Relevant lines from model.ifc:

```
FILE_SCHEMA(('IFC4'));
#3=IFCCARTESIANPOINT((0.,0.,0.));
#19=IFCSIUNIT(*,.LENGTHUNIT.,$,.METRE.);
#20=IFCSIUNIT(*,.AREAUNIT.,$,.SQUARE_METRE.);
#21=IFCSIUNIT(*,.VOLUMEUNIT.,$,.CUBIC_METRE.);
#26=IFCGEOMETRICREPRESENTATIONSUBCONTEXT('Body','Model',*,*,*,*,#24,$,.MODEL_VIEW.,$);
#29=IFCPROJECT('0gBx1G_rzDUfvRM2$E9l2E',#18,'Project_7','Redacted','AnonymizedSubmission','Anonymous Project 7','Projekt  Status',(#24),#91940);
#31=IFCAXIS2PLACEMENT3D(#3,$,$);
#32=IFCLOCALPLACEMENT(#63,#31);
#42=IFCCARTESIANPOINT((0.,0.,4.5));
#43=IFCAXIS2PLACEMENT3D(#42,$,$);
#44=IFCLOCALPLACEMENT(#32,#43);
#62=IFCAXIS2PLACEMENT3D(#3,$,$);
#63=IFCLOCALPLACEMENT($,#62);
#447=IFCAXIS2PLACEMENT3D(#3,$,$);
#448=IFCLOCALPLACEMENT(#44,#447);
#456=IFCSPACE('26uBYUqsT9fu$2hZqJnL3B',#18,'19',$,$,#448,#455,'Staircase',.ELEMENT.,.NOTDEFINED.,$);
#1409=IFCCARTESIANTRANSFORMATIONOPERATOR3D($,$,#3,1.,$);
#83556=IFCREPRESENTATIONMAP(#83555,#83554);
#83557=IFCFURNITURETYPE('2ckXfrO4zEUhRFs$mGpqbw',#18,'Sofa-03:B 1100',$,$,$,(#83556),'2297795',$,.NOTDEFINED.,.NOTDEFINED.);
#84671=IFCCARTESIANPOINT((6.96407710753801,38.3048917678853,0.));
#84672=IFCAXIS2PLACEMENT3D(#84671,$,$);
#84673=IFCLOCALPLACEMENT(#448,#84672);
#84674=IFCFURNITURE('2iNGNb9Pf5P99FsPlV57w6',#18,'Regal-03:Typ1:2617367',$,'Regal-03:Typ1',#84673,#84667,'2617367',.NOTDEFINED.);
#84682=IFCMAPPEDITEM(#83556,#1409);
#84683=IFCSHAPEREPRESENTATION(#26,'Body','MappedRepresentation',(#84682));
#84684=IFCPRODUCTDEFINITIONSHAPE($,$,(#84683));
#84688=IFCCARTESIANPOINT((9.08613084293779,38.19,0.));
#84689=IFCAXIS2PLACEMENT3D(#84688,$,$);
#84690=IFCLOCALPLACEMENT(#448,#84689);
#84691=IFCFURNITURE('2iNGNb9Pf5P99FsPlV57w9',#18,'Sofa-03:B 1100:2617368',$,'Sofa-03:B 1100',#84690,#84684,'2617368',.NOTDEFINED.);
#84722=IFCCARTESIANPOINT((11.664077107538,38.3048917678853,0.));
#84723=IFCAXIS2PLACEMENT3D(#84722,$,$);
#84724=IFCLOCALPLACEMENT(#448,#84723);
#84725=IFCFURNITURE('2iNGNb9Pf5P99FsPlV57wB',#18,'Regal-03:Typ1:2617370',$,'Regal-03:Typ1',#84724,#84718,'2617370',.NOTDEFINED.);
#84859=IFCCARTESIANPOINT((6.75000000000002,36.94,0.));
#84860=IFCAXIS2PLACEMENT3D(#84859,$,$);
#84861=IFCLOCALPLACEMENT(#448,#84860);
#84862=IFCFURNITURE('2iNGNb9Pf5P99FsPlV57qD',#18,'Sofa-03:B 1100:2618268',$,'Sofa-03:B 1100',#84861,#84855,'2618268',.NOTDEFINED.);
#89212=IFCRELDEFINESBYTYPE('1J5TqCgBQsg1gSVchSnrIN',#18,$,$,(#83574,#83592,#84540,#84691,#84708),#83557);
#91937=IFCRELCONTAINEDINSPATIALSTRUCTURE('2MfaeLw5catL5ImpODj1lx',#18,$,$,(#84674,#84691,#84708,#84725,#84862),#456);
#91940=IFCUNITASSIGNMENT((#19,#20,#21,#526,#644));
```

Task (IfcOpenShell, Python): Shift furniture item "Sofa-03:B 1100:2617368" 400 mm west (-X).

```python
import ifcopenshell
import ifcopenshell.api.geometry
import ifcopenshell.util.placement

model = ifcopenshell.open("model.ifc")

item = model.by_id(84691)
matrix = ifcopenshell.util.placement.get_local_placement(item.ObjectPlacement)
matrix[0, 3] -= 0.4
ifcopenshell.api.geometry.edit_object_placement(model, product=item, matrix=matrix, is_si=False)

print(ifcopenshell.util.placement.get_local_placement(item.ObjectPlacement).round(3) + 0.0)

model.write("model_rev.ifc")
```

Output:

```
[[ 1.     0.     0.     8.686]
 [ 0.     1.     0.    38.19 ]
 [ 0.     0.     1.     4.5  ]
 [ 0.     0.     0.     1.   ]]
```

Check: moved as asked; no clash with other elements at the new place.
